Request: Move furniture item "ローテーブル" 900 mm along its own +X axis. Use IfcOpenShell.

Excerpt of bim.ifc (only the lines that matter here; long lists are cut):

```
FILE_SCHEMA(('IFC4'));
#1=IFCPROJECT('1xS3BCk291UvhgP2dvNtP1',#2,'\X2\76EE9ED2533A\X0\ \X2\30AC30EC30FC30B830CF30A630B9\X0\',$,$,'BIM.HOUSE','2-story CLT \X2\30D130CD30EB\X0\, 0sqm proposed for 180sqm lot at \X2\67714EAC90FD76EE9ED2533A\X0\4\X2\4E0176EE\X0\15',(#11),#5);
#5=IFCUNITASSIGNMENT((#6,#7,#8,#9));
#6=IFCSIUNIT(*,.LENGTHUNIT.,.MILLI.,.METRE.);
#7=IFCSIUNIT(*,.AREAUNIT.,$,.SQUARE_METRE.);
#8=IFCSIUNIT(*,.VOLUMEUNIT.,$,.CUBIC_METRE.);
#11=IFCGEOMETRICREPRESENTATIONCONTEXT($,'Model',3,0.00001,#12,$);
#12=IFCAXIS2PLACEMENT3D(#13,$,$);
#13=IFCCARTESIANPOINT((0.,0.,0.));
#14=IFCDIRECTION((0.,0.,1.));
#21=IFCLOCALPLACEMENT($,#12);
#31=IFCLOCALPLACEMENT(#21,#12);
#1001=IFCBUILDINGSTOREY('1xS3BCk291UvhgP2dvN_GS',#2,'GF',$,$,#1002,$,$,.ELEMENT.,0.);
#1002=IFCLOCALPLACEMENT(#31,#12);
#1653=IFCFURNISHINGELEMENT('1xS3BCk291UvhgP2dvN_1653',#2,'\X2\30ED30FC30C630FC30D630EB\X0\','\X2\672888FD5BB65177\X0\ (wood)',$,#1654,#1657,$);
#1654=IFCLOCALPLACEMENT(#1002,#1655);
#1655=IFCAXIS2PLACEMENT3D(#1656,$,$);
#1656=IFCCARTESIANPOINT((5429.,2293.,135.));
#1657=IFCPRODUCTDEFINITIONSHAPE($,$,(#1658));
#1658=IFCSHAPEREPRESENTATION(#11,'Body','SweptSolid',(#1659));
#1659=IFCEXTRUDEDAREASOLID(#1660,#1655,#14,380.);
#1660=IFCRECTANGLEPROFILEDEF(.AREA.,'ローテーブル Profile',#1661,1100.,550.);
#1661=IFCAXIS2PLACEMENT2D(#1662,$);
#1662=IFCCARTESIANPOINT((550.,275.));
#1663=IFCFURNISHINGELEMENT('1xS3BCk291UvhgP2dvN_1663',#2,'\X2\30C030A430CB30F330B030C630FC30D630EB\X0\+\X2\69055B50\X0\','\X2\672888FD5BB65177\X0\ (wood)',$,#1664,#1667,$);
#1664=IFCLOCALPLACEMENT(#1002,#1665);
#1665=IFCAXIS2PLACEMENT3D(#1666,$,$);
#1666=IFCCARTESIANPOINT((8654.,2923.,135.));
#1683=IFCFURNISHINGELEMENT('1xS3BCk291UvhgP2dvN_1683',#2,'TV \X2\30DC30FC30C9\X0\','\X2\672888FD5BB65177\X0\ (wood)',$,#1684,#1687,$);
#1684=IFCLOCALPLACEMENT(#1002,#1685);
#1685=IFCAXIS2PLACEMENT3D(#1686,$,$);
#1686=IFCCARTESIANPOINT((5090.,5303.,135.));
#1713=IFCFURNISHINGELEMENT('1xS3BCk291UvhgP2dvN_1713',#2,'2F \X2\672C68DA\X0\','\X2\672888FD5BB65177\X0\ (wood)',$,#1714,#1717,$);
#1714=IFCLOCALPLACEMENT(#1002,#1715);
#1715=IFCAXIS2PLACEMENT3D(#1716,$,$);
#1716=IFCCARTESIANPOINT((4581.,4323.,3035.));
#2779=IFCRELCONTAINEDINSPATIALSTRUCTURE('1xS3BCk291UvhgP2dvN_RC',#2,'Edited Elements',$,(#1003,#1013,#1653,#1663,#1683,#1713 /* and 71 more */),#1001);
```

```python
import ifcopenshell
import ifcopenshell.api.geometry
import ifcopenshell.util.placement
import ifcopenshell.util.unit

model = ifcopenshell.open("bim.ifc")
unit_scale = ifcopenshell.util.unit.calculate_unit_scale(model)

item = model.by_guid("1xS3BCk291UvhgP2dvN_1653")
matrix = ifcopenshell.util.placement.get_local_placement(item.ObjectPlacement)
matrix[:3, 3] += matrix[:3, 0] * 0.9 / unit_scale
ifcopenshell.api.geometry.edit_object_placement(model, product=item, matrix=matrix, is_si=False)

print(ifcopenshell.util.placement.get_local_placement(item.ObjectPlacement).round(3) + 0.0)

model.write("bim_edited.ifc")
```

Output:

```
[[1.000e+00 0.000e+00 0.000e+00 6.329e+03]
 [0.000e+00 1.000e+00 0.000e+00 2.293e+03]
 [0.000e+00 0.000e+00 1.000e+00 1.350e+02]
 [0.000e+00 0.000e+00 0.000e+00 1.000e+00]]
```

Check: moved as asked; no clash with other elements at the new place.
